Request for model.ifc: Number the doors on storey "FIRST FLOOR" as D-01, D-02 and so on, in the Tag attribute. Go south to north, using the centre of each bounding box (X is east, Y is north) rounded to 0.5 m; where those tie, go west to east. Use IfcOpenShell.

First a look at what the model holds.

```python
import ifcopenshell
import ifcopenshell.util.element
import ifcopenshell.util.placement

model = ifcopenshell.open("model.ifc")
print(model.schema)
storey = next(s for s in model.by_type("IfcBuildingStorey") if s.Name == "FIRST FLOOR")
doors = [e for e in ifcopenshell.util.element.get_decomposition(storey) if e.is_a("IfcDoor")]
for e in sorted(doors, key=lambda e: e.id()):
    origin = ifcopenshell.util.placement.get_local_placement(e.ObjectPlacement)[:3, 3]
    print(e.id(), e.Tag, e.Name, origin.round(2) + 0.0, sep=" | ")
```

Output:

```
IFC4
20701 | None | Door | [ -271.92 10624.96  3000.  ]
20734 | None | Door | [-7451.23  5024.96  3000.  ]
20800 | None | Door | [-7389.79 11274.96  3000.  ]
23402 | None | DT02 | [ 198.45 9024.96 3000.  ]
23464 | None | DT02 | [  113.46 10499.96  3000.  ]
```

```python
import ifcopenshell
import ifcopenshell.geom
import ifcopenshell.util.element
import ifcopenshell.util.shape

model = ifcopenshell.open("model.ifc")
settings = ifcopenshell.geom.settings()
settings.set("use-world-coords", True)


def centre(element):
    shape = ifcopenshell.geom.create_shape(settings, element)
    return ifcopenshell.util.shape.get_bbox_centroid(shape.geometry)


storey = next(s for s in model.by_type("IfcBuildingStorey") if s.Name == "FIRST FLOOR")
doors = [e for e in ifcopenshell.util.element.get_decomposition(storey) if e.is_a("IfcDoor")]

# Insertion points can sit at a corner or the storey origin, so sort by the geometry (in metres).
centres = {e: centre(e) for e in doors}
doors.sort(key=lambda e: (round(centres[e][1] / 0.5), centres[e][0]))

for i, e in enumerate(doors, start=1):
    number = f"D-{i:02d}"
    e.Tag = number
    print(e.id(), number)

model.write("model_v2.ifc")
```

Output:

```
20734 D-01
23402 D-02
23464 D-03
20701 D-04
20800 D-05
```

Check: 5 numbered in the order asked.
